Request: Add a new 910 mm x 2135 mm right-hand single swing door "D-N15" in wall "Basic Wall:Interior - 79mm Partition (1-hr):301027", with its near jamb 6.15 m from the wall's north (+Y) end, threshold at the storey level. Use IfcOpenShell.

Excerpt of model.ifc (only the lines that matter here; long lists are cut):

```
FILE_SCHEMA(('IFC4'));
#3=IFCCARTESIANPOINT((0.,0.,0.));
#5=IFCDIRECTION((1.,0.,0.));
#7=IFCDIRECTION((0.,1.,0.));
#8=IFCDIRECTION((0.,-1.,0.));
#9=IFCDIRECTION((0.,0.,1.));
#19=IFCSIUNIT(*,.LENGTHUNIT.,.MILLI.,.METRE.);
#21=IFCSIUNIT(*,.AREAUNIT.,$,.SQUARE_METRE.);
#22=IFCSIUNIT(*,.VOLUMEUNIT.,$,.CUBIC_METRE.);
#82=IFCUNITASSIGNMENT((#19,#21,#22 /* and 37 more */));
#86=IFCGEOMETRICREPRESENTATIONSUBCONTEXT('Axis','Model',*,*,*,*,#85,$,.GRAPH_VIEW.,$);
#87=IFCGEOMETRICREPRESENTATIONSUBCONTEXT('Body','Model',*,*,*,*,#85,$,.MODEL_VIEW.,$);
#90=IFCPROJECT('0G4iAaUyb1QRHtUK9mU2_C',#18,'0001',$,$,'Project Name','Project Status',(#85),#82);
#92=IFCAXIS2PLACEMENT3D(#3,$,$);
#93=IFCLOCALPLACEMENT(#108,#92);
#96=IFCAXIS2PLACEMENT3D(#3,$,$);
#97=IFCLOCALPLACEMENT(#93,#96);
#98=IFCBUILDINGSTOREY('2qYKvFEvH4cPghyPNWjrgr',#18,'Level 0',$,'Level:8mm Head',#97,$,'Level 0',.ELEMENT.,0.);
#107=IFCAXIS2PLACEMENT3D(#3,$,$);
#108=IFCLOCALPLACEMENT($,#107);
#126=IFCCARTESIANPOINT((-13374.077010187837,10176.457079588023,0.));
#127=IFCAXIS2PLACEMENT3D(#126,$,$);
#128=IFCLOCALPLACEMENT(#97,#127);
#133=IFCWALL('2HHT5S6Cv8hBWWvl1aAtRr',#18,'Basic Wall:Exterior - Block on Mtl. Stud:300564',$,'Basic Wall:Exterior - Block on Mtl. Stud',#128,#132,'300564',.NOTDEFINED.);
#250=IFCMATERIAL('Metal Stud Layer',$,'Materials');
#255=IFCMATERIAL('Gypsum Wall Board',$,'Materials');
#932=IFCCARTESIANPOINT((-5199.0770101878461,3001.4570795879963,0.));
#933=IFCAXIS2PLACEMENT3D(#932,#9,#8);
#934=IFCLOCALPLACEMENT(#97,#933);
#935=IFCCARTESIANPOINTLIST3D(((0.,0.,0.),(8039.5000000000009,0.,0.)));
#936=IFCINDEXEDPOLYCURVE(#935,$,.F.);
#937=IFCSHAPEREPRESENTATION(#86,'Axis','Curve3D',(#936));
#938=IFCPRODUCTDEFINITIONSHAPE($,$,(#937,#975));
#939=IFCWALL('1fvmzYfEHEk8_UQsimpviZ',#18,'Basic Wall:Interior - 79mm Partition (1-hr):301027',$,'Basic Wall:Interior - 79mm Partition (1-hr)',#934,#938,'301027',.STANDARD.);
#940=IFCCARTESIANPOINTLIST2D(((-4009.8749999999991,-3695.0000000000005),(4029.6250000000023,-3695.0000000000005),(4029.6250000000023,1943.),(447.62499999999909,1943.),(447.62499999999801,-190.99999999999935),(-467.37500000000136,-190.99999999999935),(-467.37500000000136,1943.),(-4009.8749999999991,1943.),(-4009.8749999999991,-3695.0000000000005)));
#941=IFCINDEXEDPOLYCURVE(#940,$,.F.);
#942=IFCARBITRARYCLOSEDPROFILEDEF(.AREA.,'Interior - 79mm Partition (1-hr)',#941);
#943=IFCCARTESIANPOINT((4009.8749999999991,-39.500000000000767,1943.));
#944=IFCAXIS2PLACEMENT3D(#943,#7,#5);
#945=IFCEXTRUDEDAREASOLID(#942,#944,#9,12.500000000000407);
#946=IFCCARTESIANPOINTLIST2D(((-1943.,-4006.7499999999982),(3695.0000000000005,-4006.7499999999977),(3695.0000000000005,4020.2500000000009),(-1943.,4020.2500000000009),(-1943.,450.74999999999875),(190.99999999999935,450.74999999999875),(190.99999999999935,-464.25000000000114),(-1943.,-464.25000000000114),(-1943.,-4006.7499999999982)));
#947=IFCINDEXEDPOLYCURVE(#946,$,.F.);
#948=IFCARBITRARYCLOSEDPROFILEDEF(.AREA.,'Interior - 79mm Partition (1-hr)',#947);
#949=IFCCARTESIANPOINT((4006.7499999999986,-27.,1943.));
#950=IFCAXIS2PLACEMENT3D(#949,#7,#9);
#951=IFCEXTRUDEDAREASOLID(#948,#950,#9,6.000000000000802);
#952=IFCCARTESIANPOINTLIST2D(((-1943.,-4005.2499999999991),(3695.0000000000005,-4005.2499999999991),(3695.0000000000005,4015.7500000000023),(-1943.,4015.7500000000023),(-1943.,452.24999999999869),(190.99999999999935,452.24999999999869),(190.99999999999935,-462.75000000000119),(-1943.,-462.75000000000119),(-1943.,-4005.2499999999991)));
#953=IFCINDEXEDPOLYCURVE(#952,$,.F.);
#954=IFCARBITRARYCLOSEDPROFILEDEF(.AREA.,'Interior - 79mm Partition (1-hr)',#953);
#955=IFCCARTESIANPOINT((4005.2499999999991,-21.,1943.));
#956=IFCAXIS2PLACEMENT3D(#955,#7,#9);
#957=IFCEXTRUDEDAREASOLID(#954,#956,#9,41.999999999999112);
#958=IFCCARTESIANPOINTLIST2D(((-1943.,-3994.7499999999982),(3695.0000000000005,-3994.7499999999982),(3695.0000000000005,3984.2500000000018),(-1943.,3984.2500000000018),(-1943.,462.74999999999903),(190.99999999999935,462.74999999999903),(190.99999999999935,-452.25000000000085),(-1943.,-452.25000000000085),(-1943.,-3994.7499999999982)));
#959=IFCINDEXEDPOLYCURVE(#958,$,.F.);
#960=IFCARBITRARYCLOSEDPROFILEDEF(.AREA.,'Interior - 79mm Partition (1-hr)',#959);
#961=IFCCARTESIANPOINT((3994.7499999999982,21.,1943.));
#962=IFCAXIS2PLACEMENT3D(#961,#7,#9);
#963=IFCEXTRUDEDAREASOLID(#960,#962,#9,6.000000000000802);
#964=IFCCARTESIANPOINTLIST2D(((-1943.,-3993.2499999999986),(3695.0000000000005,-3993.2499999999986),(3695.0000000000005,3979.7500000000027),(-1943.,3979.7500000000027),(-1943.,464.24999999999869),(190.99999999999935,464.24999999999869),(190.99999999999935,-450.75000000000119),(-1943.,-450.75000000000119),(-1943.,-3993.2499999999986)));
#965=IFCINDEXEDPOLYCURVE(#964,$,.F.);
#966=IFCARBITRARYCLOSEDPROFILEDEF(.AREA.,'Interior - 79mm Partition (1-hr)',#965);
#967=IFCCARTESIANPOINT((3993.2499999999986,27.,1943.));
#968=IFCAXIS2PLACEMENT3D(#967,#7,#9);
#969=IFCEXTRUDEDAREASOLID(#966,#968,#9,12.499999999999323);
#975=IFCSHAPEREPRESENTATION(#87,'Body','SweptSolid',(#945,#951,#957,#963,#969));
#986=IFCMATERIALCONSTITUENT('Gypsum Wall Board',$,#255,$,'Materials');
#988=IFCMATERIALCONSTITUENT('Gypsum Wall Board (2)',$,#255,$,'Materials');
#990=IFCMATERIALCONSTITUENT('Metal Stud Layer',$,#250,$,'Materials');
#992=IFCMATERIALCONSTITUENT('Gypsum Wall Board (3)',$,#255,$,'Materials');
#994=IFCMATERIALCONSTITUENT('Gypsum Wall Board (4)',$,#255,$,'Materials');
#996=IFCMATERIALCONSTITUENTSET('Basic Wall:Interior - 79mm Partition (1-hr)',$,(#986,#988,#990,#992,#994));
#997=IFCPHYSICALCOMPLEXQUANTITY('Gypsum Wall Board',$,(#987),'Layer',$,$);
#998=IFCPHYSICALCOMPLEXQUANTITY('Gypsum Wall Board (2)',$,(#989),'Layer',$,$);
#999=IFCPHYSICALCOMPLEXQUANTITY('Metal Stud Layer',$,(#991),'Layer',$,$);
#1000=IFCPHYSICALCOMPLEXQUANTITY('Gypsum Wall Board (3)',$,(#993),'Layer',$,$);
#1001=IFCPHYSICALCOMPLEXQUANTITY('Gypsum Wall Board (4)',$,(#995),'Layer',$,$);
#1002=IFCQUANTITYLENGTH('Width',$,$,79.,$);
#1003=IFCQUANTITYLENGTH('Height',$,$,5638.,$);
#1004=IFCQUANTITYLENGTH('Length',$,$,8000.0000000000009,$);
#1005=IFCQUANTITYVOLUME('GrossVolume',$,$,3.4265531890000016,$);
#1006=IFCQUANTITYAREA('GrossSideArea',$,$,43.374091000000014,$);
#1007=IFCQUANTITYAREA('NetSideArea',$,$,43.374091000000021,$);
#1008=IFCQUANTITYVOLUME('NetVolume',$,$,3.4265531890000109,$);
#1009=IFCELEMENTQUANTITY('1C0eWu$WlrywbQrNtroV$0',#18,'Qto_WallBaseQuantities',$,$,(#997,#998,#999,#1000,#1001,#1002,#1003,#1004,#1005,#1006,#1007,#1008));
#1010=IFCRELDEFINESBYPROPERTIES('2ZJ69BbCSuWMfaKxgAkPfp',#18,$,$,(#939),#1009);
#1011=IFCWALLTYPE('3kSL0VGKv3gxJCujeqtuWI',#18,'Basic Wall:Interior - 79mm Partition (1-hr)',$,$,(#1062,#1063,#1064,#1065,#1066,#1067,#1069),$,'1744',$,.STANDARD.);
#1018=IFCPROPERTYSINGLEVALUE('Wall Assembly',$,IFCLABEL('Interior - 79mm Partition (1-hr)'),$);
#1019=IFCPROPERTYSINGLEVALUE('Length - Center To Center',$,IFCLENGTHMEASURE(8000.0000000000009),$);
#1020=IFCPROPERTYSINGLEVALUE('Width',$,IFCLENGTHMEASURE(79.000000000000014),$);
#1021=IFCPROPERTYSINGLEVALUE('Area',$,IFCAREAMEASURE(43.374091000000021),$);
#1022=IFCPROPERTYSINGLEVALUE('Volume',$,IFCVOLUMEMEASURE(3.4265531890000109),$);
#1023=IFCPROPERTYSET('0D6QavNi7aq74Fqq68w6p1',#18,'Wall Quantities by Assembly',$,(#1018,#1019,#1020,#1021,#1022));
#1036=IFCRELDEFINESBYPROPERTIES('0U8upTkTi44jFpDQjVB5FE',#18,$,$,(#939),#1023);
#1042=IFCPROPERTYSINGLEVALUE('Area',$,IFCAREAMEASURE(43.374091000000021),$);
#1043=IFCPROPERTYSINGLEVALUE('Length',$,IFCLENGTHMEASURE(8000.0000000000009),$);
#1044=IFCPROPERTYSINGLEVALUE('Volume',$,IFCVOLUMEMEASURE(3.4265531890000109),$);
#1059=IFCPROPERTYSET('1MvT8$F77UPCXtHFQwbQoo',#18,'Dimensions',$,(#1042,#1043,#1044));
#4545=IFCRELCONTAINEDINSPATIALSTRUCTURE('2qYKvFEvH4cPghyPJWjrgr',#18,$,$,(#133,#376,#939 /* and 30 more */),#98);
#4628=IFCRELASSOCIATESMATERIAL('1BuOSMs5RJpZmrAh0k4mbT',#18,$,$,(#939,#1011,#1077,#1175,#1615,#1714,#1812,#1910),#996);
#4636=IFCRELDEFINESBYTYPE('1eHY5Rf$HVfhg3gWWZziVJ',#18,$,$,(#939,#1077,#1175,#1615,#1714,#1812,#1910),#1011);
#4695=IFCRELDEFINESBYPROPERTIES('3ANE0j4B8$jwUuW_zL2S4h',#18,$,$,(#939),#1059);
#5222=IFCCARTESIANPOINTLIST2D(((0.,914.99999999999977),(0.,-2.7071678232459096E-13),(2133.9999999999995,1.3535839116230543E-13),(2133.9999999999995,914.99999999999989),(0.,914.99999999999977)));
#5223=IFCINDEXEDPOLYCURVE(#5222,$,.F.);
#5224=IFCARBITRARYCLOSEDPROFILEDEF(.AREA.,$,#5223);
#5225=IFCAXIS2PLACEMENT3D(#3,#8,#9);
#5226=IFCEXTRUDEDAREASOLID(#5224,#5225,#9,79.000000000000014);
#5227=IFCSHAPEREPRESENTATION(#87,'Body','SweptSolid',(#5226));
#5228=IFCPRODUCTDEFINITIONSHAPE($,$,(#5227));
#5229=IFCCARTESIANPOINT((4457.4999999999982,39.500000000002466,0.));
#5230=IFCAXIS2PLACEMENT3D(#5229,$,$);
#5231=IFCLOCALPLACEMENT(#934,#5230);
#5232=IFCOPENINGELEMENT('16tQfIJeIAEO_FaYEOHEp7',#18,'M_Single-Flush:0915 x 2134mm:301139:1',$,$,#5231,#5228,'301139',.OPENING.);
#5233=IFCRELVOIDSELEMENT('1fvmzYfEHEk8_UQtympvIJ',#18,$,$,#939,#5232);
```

```python
import numpy as np
import ifcopenshell
import ifcopenshell.api.feature
import ifcopenshell.api.geometry
import ifcopenshell.api.pset
import ifcopenshell.api.root
import ifcopenshell.api.spatial
import ifcopenshell.geom
import ifcopenshell.util.element
import ifcopenshell.util.placement
import ifcopenshell.util.representation
import ifcopenshell.util.shape
import ifcopenshell.util.unit

model = ifcopenshell.open("model.ifc")
unit_scale = ifcopenshell.util.unit.calculate_unit_scale(model)
area_scale = ifcopenshell.util.unit.calculate_unit_scale(model, "AREAUNIT")
volume_scale = ifcopenshell.util.unit.calculate_unit_scale(model, "VOLUMEUNIT")
settings = ifcopenshell.geom.settings()


def volume(element):
    """Net volume in cubic metres, openings subtracted."""
    shape = ifcopenshell.geom.create_shape(settings, element)
    return ifcopenshell.util.shape.get_volume(shape.geometry)


wall = model.by_guid("1fvmzYfEHEk8_UQsimpviZ")
storey = ifcopenshell.util.element.get_container(wall, ifc_class="IfcBuildingStorey")
context = ifcopenshell.util.representation.get_context(model, "Model", "Body", "MODEL_VIEW")
before = volume(wall)

width, height, from_end, sill = 0.91, 2.135, 6.15, 0.0  # metres

# The wall runs along its own X axis, and the end named is its -X end.
wall_shape = ifcopenshell.geom.create_shape(settings, wall)
x, y, z = ifcopenshell.util.shape.get_vertices(wall_shape.geometry).T
start = x.min() + from_end
face, thickness = float(y.min()), float(y.max() - y.min())
wall_matrix = ifcopenshell.util.placement.get_local_placement(wall.ObjectPlacement)
level = ifcopenshell.util.placement.get_local_placement(storey.ObjectPlacement)[2, 3]


def in_wall(x, y):
    """Placement at x, y metres in the wall's axes, at sill height."""
    matrix = wall_matrix.copy()
    matrix[:, 3] = wall_matrix @ np.array([x / unit_scale, y / unit_scale, 0.0, 1.0])
    matrix[2, 3] = level + sill / unit_scale
    return matrix


# Opening: a box that overshoots both wall faces by 50 mm.
opening = ifcopenshell.api.root.create_entity(model, ifc_class="IfcOpeningElement", predefined_type="OPENING")
box = ifcopenshell.api.geometry.add_wall_representation(
    model, context=context, length=width, height=height, thickness=thickness + 0.1
)
ifcopenshell.api.geometry.assign_representation(model, product=opening, representation=box)
ifcopenshell.api.geometry.edit_object_placement(model, product=opening, matrix=in_wall(start, face - 0.05), is_si=False)
ifcopenshell.api.feature.add_feature(model, feature=opening, element=wall)

door = ifcopenshell.api.root.create_entity(model, ifc_class="IfcDoor", name="D-N15", predefined_type="DOOR")
door.OverallWidth, door.OverallHeight = width / unit_scale, height / unit_scale
door.OperationType = "SINGLE_SWING_RIGHT"
body = ifcopenshell.api.geometry.add_door_representation(
    model,
    context=context,
    overall_width=door.OverallWidth,
    overall_height=door.OverallHeight,
    operation_type="SINGLE_SWING_RIGHT",
    lining_properties={"LiningDepth": thickness / unit_scale, "ThresholdDepth": thickness / unit_scale},
)
ifcopenshell.api.geometry.assign_representation(model, product=door, representation=body)
ifcopenshell.api.spatial.assign_container(model, products=[door], relating_structure=storey)
ifcopenshell.api.feature.add_filling(model, opening=opening, element=door)

# The lining spans the wall, so the door starts at the wall face.
ifcopenshell.api.geometry.edit_object_placement(model, product=door, matrix=in_wall(start, face), is_si=False)

after = volume(wall)

# Update the wall's stored quantities.
qto = model.by_id(ifcopenshell.util.element.get_pset(wall, "Qto_WallBaseQuantities", should_inherit=False)["id"])
ifcopenshell.api.pset.edit_qto(model, qto=qto, properties={
    "NetSideArea": after / thickness / area_scale,
    "NetVolume": after / volume_scale,
})
pset = model.by_id(ifcopenshell.util.element.get_pset(wall, "Wall Quantities by Assembly", should_inherit=False)["id"])
ifcopenshell.api.pset.edit_pset(model, pset=pset, properties={
    "Area": model.create_entity("IfcAreaMeasure", after / thickness / area_scale),
    "Volume": model.create_entity("IfcVolumeMeasure", after / volume_scale),
})
pset = model.by_id(ifcopenshell.util.element.get_pset(wall, "Dimensions", should_inherit=False)["id"])
ifcopenshell.api.pset.edit_pset(model, pset=pset, properties={
    "Area": model.create_entity("IfcAreaMeasure", after / thickness / area_scale),
    "Volume": model.create_entity("IfcVolumeMeasure", after / volume_scale),
})

print(f"wall volume {before:.3f} -> {after:.3f} m3")

model.write("model_v2.ifc")
```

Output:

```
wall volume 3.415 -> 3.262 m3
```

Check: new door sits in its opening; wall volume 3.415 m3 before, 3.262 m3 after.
